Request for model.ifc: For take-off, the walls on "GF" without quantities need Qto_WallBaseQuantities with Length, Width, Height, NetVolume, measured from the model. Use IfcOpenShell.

First a look at what the model holds.

```python
import ifcopenshell
import ifcopenshell.util.element
import ifcopenshell.util.unit

model = ifcopenshell.open("model.ifc")
print(model.schema)
for unit_type in ("LENGTHUNIT", "AREAUNIT", "VOLUMEUNIT"):
    print(unit_type, ifcopenshell.util.unit.calculate_unit_scale(model, unit_type))
storey = next(s for s in model.by_type("IfcBuildingStorey") if s.Name == "GF")
walls = [e for e in ifcopenshell.util.element.get_decomposition(storey) if e.is_a("IfcWall")]
for e in sorted(walls, key=lambda e: e.id()):
    print(e.id(), e.is_a(), e.Name, list(ifcopenshell.util.element.get_psets(e, qtos_only=True)), sep=" | ")
```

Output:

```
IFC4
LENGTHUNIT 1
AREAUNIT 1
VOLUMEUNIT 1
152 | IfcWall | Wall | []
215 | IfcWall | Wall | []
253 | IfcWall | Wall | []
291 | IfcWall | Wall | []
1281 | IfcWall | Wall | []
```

```python
import ifcopenshell
import ifcopenshell.api.pset
import ifcopenshell.geom
import ifcopenshell.util.element
import ifcopenshell.util.shape
import ifcopenshell.util.unit

model = ifcopenshell.open("model.ifc")
unit_scale = ifcopenshell.util.unit.calculate_unit_scale(model)
volume_scale = ifcopenshell.util.unit.calculate_unit_scale(model, "VOLUMEUNIT")
settings = ifcopenshell.geom.settings()

storey = next(s for s in model.by_type("IfcBuildingStorey") if s.Name == "GF")
walls = [e for e in ifcopenshell.util.element.get_decomposition(storey) if e.is_a("IfcWall")]

for e in sorted(walls, key=lambda e: e.id()):
    if ifcopenshell.util.element.get_psets(e, qtos_only=True, should_inherit=False):
        continue
    # Geometry comes back in metres, in the element's own axes.
    shape = ifcopenshell.geom.create_shape(settings, e)
    values = {
        "Length": ifcopenshell.util.shape.get_x(shape.geometry) / unit_scale,
        "Width": ifcopenshell.util.shape.get_y(shape.geometry) / unit_scale,
        "Height": ifcopenshell.util.shape.get_z(shape.geometry) / unit_scale,
        "NetVolume": ifcopenshell.util.shape.get_volume(shape.geometry) / volume_scale,
    }
    qto = ifcopenshell.api.pset.add_qto(model, product=e, name="Qto_WallBaseQuantities")
    ifcopenshell.api.pset.edit_qto(model, qto=qto, properties=values)
    print(e.id(), {k: round(v, 3) for k, v in values.items()})

model.write("model_updated.ifc")
```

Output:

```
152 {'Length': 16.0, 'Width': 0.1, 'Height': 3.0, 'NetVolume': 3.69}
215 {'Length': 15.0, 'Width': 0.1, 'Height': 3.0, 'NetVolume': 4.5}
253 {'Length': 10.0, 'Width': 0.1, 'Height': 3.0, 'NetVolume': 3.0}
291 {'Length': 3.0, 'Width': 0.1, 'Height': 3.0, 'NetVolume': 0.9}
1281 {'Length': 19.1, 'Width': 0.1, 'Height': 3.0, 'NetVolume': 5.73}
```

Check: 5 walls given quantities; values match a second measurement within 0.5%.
